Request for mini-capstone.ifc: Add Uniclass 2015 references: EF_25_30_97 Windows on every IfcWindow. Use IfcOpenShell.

First a look at what the model holds.

```python
import ifcopenshell

model = ifcopenshell.open("mini-capstone.ifc")
print(model.schema)
print("classifications:", [c.Name for c in model.by_type("IfcClassification")])
for ifc_class in ("IfcDoor", "IfcRoof", "IfcStair", "IfcWall", "IfcWindow"):
    print(ifc_class, len(model.by_type(ifc_class)))
```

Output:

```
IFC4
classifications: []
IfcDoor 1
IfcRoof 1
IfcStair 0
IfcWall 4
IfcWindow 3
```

```python
import ifcopenshell
import ifcopenshell.api.classification

model = ifcopenshell.open("mini-capstone.ifc")

system = ifcopenshell.api.classification.add_classification(model, classification="Uniclass 2015")

codes = {
    "IfcWindow": ("EF_25_30_97", "Windows"),
}
for ifc_class, (code, name) in codes.items():
    products = model.by_type(ifc_class)
    ifcopenshell.api.classification.add_reference(
        model, products=products, classification=system, identification=code, name=name
    )
    print(code, len(products))

model.write("mini-capstone_edited.ifc")
```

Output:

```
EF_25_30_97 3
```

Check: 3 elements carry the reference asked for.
